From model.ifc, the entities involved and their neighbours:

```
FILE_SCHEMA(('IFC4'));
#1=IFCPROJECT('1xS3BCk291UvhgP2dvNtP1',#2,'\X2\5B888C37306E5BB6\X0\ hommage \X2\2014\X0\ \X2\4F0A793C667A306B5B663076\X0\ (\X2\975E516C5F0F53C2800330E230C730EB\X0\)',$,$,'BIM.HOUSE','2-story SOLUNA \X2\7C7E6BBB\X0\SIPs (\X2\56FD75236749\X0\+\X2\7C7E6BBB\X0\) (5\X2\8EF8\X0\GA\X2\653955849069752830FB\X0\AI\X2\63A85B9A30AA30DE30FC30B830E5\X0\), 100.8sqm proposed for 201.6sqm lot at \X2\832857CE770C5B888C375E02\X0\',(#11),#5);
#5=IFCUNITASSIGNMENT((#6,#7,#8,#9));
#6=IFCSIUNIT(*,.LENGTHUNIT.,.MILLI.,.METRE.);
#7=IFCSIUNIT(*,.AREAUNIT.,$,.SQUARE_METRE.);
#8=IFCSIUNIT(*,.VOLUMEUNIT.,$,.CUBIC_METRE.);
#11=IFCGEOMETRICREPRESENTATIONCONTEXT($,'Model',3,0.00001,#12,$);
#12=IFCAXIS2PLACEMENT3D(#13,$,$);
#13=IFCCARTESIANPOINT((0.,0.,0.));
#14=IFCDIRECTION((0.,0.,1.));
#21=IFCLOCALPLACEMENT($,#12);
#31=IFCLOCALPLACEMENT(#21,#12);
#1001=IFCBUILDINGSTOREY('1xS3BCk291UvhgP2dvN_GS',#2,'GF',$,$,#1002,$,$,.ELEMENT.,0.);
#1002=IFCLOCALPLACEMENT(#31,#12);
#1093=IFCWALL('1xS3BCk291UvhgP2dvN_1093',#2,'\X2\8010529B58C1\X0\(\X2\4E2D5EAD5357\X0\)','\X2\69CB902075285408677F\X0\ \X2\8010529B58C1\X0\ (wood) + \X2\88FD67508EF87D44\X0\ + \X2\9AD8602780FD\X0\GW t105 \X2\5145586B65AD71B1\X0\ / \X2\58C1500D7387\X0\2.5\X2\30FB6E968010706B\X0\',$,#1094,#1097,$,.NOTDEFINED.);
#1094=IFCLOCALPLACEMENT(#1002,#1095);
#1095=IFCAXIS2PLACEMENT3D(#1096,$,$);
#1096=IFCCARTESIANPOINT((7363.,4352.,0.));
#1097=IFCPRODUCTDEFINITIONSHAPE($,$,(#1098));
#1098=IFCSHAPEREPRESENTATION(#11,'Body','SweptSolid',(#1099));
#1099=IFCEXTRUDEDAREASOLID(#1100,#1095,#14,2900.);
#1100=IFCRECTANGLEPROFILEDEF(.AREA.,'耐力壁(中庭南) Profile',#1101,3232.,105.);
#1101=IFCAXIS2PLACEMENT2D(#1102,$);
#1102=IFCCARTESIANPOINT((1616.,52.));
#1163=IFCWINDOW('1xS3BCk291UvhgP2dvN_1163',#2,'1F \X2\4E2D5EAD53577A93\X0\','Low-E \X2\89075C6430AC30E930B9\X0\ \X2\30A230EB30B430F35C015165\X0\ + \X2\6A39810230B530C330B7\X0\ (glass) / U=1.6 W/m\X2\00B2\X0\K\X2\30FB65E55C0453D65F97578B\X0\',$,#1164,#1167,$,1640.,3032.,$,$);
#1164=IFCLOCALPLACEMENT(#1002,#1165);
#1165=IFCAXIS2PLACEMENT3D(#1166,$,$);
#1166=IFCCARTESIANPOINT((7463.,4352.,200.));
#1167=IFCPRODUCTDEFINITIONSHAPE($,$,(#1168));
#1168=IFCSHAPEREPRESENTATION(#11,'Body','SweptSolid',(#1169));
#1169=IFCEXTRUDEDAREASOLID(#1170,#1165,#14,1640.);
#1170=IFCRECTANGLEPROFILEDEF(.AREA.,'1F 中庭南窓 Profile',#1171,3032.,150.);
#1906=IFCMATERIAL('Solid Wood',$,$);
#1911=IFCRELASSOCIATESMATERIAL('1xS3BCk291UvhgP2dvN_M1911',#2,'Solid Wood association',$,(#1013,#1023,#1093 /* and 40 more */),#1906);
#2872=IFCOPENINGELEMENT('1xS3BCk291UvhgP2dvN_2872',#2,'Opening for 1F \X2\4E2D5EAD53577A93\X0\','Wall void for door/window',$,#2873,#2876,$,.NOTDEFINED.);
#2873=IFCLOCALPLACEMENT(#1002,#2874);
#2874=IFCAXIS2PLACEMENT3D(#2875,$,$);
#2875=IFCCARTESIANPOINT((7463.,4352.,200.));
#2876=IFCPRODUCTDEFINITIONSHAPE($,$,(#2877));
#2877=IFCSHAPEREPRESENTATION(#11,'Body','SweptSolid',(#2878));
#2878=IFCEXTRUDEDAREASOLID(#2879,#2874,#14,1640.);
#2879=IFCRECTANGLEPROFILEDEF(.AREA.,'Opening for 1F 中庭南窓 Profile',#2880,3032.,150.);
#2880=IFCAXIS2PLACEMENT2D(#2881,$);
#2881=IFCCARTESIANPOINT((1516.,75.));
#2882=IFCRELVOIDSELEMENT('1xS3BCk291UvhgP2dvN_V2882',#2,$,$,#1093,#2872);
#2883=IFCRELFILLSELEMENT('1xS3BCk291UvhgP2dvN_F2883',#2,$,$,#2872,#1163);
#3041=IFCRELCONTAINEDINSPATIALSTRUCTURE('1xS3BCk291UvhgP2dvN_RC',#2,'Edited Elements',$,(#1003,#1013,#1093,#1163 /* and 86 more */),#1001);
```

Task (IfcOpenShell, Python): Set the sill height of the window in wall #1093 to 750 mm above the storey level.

```python
import numpy as np
import ifcopenshell
import ifcopenshell.api.geometry
import ifcopenshell.geom
import ifcopenshell.util.element
import ifcopenshell.util.placement
import ifcopenshell.util.shape
import ifcopenshell.util.unit

model = ifcopenshell.open("model.ifc")
unit_scale = ifcopenshell.util.unit.calculate_unit_scale(model)

window = model.by_guid("1xS3BCk291UvhgP2dvN_1163")
opening = window.FillsVoids[0].RelatingOpeningElement
storey = ifcopenshell.util.element.get_container(window, ifc_class="IfcBuildingStorey")
level = ifcopenshell.util.placement.get_local_placement(storey.ObjectPlacement)[2, 3]

# The opening's origin need not be at the sill, so measure its lowest point.
shape = ifcopenshell.geom.create_shape(ifcopenshell.geom.settings(), opening)
bottom = ifcopenshell.util.shape.get_shape_bottom_elevation(shape, shape.geometry) / unit_scale
dz = level + 750.0 - bottom

shift = np.array([0.0, 0.0, dz])
# The window is not placed relative to its opening, so move both.
for product in (opening, window):
    matrix = ifcopenshell.util.placement.get_local_placement(product.ObjectPlacement)
    matrix[:3, 3] += shift
    ifcopenshell.api.geometry.edit_object_placement(model, product=product, matrix=matrix, is_si=False)

print(f"moved by {dz * unit_scale:+.3f} m")

model.write("model_edited.ifc")
```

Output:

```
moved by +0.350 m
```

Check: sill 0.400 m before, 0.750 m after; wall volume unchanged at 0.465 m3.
